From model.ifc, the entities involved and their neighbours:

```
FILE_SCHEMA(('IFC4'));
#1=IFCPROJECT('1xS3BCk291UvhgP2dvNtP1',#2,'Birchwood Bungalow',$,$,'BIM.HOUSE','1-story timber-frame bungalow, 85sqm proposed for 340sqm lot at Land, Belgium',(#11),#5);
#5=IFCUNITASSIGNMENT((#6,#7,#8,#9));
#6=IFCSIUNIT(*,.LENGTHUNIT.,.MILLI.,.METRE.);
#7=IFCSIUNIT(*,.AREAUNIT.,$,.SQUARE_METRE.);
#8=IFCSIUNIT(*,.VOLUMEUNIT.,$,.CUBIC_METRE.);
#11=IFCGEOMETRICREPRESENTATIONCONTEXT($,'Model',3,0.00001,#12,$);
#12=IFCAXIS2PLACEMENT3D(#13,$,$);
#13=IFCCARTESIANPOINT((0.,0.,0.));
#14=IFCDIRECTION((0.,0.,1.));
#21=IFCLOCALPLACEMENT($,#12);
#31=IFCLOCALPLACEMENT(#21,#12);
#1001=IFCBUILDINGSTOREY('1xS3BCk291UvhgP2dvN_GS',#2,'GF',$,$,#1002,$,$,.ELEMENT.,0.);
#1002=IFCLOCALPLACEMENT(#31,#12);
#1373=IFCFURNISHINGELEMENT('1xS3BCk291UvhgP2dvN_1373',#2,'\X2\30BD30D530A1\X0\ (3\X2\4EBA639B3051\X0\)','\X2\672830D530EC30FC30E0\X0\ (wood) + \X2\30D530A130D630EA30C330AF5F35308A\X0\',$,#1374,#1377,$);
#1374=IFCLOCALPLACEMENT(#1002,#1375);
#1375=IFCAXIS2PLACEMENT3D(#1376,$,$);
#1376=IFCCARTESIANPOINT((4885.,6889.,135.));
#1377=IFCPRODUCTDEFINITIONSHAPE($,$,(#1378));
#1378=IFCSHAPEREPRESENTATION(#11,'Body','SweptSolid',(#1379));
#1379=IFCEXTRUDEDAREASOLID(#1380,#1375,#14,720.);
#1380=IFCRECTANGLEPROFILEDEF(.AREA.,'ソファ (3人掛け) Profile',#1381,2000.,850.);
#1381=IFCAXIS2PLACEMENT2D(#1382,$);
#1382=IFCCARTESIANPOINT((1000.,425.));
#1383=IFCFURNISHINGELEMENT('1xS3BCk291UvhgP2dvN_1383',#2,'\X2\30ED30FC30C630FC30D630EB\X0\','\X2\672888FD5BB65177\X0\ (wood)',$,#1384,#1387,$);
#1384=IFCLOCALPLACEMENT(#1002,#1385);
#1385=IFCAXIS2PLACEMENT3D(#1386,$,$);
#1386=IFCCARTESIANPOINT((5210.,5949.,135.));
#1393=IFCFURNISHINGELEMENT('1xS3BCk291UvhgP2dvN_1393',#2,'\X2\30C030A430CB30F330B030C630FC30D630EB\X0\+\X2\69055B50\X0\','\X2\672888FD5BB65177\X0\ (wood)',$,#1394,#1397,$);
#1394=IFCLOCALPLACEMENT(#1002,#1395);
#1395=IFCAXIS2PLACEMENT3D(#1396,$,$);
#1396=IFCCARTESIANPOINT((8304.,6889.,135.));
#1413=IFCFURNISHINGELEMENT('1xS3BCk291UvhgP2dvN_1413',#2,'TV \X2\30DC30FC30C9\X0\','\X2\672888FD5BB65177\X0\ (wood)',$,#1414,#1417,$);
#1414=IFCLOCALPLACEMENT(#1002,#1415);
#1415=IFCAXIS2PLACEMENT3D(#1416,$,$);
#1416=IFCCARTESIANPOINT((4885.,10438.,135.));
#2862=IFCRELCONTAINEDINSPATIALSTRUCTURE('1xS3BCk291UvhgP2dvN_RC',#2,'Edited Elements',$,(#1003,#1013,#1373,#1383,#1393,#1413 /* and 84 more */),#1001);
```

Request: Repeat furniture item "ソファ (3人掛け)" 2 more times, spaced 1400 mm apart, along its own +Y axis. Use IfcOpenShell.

```python
import ifcopenshell
import ifcopenshell.api.geometry
import ifcopenshell.api.root
import ifcopenshell.util.element
import ifcopenshell.util.placement

model = ifcopenshell.open("model.ifc")


def reuse_history(source, copy):
    """copy_class also copies each property set's owner history, people and application; keep the originals."""
    for rel in copy.IsDefinedBy:
        if rel.is_a("IfcRelDefinesByProperties") and (history := rel.RelatingPropertyDefinition.OwnerHistory):
            rel.RelatingPropertyDefinition.OwnerHistory = source.OwnerHistory
            ifcopenshell.util.element.remove_deep2(model, history)


source = model.by_guid("1xS3BCk291UvhgP2dvN_1373")
base = ifcopenshell.util.placement.get_local_placement(source.ObjectPlacement)
step = base[:3, 1] * 1400.0

for i in range(1, 3):
    copy = ifcopenshell.api.root.copy_class(model, product=source)
    copy.Representation = ifcopenshell.util.element.copy_deep(
        model, source.Representation, exclude=["IfcGeometricRepresentationContext", "IfcRepresentationMap"]
    )
    reuse_history(source, copy)
    matrix = base.copy()
    matrix[:3, 3] += i * step
    print("added at", matrix[:3, 3].round(3) + 0.0)
    ifcopenshell.api.geometry.edit_object_placement(model, product=copy, matrix=matrix, is_si=False)

model.write("model_edited.ifc")
```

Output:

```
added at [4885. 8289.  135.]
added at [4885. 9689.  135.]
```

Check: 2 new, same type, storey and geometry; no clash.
